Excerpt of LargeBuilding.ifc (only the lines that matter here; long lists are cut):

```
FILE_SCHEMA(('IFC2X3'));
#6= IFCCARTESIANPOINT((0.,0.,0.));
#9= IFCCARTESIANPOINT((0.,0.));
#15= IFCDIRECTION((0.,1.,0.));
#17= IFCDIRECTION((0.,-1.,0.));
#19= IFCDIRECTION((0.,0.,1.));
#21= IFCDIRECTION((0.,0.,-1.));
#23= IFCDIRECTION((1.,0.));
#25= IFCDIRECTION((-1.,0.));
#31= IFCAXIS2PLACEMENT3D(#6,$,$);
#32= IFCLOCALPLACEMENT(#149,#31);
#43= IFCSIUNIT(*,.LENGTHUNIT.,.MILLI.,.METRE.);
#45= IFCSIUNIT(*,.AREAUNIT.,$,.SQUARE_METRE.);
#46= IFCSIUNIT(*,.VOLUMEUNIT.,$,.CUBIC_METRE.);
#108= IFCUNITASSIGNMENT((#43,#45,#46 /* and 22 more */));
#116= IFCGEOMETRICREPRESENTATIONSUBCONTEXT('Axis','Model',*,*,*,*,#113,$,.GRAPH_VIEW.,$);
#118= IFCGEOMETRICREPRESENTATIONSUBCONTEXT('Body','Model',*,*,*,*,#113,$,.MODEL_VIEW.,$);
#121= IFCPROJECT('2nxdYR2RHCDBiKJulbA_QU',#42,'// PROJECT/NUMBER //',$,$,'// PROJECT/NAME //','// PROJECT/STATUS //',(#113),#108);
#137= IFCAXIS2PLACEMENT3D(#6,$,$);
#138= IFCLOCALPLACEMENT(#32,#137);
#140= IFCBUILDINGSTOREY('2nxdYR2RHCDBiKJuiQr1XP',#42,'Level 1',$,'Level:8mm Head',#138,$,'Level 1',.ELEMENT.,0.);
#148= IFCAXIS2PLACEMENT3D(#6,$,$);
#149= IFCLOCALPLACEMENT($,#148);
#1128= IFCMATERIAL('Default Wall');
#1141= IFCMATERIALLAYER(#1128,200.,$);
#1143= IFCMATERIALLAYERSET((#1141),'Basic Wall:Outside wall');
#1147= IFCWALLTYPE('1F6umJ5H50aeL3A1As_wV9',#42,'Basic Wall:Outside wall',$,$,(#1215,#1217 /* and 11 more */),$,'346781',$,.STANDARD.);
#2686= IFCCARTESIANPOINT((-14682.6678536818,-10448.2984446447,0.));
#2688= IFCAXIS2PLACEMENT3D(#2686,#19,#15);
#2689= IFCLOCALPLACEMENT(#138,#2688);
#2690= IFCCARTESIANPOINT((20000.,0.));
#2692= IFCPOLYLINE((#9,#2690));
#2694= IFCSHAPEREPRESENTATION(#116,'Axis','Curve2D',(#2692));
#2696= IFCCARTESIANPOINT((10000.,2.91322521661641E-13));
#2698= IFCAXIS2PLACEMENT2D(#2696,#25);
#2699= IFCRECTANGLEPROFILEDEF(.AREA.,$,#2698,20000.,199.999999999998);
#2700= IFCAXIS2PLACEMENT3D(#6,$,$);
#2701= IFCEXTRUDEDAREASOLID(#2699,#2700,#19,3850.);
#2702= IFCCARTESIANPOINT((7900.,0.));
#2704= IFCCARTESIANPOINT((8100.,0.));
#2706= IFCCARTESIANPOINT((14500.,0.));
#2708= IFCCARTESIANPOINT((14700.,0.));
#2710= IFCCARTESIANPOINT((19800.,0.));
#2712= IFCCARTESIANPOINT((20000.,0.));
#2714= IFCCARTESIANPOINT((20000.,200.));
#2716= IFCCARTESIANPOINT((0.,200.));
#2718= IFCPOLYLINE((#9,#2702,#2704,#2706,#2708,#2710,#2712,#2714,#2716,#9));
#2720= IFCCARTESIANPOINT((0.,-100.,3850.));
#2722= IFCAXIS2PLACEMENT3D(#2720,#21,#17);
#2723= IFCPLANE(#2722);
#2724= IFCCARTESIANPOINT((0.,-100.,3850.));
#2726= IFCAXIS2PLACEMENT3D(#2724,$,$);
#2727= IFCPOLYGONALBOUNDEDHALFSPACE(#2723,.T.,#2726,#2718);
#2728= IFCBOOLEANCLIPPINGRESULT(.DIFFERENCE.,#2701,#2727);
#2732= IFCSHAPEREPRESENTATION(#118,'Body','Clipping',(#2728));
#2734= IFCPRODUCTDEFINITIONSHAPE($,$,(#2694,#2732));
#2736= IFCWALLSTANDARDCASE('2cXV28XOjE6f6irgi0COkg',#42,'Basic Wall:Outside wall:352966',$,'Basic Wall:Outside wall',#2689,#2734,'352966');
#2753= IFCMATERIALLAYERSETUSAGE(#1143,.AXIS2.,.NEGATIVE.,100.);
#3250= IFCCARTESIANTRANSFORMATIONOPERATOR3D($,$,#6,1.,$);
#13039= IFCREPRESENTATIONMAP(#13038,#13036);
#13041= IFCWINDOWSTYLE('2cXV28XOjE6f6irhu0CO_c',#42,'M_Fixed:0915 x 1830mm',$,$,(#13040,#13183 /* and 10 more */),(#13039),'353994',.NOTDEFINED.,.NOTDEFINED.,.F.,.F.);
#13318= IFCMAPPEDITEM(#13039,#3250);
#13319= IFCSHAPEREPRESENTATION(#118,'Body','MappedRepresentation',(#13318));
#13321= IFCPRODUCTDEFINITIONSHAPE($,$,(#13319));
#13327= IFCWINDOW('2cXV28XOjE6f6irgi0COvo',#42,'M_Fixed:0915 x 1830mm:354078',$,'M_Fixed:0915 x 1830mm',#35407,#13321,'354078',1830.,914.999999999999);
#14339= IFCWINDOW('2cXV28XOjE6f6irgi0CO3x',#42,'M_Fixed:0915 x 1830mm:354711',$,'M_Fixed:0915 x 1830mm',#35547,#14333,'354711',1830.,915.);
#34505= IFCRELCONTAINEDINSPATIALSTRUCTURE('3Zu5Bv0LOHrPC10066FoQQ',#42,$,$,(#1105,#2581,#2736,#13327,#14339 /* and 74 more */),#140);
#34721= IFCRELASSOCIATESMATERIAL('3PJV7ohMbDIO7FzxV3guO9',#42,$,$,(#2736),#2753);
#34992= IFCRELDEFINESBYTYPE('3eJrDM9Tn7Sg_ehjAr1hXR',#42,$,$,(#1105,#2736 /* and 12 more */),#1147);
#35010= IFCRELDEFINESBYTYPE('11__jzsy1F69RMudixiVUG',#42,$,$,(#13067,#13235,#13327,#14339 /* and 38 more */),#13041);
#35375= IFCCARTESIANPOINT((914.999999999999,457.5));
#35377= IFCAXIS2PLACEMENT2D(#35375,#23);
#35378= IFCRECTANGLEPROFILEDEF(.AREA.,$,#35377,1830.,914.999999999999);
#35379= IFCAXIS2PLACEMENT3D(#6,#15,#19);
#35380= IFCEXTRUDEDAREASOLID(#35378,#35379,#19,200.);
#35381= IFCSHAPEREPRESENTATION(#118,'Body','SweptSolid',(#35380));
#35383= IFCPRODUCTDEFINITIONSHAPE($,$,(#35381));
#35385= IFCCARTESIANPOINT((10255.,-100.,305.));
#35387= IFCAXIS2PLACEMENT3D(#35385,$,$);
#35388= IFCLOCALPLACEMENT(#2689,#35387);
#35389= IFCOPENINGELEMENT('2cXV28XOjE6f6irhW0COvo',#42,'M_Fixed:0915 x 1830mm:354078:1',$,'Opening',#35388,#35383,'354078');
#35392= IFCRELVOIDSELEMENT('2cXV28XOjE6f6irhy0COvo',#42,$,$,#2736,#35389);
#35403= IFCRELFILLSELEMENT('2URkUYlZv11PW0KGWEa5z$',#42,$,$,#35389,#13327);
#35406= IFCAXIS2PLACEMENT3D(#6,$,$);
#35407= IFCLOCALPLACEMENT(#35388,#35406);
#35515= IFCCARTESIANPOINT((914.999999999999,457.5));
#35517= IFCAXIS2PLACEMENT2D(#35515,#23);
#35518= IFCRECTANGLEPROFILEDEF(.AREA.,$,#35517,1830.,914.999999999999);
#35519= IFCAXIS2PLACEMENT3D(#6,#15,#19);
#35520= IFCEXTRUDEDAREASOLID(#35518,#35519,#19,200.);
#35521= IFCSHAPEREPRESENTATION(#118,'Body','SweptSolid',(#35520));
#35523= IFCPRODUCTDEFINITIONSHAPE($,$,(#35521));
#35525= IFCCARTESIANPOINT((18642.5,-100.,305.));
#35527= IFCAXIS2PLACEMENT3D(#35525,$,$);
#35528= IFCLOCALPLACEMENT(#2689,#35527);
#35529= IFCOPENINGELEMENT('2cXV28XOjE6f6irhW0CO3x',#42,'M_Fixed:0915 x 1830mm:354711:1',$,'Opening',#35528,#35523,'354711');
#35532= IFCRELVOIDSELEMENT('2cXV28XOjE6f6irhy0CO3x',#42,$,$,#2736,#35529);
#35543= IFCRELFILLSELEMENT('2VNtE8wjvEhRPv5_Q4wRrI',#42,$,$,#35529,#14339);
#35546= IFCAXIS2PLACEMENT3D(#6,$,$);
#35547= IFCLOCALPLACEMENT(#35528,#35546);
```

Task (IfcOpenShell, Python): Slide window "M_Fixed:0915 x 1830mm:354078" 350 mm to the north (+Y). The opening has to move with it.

```python
import ifcopenshell
import ifcopenshell.api.geometry
import ifcopenshell.util.placement
import ifcopenshell.util.unit

model = ifcopenshell.open("LargeBuilding.ifc")
unit_scale = ifcopenshell.util.unit.calculate_unit_scale(model)

window = model.by_guid("2cXV28XOjE6f6irgi0COvo")
opening = window.FillsVoids[0].RelatingOpeningElement
wall = opening.VoidsElements[0].RelatingBuildingElement

wall_matrix = ifcopenshell.util.placement.get_local_placement(wall.ObjectPlacement)
shift = wall_matrix[:3, 0] * 0.35 / unit_scale
before = ifcopenshell.util.placement.get_local_placement(window.ObjectPlacement)[:3, 3].copy()

# The window is placed relative to its opening, so it follows when the opening moves.
matrix = ifcopenshell.util.placement.get_local_placement(opening.ObjectPlacement)
matrix[:3, 3] += shift
ifcopenshell.api.geometry.edit_object_placement(
    model, product=opening, matrix=matrix, is_si=False, should_transform_children=True
)

after = ifcopenshell.util.placement.get_local_placement(window.ObjectPlacement)[:3, 3]
print("window moved by", (after - before).round(3) + 0.0)

model.write("LargeBuilding_updated.ifc")
```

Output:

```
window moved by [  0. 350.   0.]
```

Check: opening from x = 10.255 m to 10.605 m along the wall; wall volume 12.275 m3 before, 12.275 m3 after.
